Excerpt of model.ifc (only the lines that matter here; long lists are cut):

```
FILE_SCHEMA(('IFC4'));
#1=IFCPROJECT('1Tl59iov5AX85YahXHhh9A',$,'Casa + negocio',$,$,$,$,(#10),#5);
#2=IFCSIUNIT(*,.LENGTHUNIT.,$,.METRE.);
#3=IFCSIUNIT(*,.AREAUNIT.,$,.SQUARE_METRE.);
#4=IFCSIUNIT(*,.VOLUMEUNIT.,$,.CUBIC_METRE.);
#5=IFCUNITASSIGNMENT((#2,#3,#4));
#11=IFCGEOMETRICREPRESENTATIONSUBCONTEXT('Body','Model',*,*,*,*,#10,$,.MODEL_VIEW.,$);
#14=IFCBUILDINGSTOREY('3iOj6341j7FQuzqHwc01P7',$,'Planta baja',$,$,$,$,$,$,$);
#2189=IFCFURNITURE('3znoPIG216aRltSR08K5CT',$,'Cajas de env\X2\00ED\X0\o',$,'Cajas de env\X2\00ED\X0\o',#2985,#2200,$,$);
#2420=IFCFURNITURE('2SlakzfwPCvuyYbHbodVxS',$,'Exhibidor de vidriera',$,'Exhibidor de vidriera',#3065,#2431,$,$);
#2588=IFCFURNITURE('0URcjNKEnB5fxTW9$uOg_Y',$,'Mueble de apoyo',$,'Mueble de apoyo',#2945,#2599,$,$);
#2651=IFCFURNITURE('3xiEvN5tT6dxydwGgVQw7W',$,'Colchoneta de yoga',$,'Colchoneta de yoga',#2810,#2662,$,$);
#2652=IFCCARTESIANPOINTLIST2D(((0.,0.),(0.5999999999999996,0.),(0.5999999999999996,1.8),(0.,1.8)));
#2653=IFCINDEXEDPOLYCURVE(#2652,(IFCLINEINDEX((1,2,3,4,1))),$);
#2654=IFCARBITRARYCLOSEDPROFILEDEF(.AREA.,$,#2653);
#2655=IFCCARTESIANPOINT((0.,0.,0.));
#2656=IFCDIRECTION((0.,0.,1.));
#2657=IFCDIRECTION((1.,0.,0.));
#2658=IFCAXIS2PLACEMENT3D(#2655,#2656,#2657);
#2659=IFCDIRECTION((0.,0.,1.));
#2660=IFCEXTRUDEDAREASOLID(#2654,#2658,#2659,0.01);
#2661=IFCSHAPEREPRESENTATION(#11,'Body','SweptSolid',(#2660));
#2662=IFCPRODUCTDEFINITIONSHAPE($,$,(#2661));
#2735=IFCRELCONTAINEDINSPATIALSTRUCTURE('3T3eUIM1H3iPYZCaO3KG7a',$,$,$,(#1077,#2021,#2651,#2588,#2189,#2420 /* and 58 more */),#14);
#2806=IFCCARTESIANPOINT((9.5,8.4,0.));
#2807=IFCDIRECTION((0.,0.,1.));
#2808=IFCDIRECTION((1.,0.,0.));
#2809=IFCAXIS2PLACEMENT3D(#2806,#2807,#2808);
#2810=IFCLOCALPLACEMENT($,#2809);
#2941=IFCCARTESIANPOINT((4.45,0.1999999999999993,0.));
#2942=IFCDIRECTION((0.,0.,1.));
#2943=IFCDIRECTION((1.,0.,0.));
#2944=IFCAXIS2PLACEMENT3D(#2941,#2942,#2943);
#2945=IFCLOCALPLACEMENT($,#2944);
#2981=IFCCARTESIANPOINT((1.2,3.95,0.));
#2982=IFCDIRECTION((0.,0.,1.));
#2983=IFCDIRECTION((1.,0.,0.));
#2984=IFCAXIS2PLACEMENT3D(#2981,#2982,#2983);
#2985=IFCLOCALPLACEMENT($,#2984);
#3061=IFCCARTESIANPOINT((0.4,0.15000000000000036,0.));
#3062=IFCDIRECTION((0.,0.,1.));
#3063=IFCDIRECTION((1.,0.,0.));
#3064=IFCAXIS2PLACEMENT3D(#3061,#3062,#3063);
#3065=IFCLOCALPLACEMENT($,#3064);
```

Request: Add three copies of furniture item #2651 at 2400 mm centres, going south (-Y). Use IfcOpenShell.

```python
import numpy as np
import ifcopenshell
import ifcopenshell.api.geometry
import ifcopenshell.api.root
import ifcopenshell.util.element
import ifcopenshell.util.placement

model = ifcopenshell.open("model.ifc")

source = model.by_guid("3xiEvN5tT6dxydwGgVQw7W")
base = ifcopenshell.util.placement.get_local_placement(source.ObjectPlacement)
step = np.array([0.0, -1.0, 0.0]) * 2.4

for i in range(1, 4):
    copy = ifcopenshell.api.root.copy_class(model, product=source)
    copy.Representation = ifcopenshell.util.element.copy_deep(
        model, source.Representation, exclude=["IfcGeometricRepresentationContext", "IfcRepresentationMap"]
    )
    matrix = base.copy()
    matrix[:3, 3] += i * step
    print("added at", matrix[:3, 3].round(3) + 0.0)
    ifcopenshell.api.geometry.edit_object_placement(model, product=copy, matrix=matrix, is_si=False)

model.write("model_updated.ifc")
```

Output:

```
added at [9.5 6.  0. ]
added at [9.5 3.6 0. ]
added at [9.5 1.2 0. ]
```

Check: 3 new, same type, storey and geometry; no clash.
